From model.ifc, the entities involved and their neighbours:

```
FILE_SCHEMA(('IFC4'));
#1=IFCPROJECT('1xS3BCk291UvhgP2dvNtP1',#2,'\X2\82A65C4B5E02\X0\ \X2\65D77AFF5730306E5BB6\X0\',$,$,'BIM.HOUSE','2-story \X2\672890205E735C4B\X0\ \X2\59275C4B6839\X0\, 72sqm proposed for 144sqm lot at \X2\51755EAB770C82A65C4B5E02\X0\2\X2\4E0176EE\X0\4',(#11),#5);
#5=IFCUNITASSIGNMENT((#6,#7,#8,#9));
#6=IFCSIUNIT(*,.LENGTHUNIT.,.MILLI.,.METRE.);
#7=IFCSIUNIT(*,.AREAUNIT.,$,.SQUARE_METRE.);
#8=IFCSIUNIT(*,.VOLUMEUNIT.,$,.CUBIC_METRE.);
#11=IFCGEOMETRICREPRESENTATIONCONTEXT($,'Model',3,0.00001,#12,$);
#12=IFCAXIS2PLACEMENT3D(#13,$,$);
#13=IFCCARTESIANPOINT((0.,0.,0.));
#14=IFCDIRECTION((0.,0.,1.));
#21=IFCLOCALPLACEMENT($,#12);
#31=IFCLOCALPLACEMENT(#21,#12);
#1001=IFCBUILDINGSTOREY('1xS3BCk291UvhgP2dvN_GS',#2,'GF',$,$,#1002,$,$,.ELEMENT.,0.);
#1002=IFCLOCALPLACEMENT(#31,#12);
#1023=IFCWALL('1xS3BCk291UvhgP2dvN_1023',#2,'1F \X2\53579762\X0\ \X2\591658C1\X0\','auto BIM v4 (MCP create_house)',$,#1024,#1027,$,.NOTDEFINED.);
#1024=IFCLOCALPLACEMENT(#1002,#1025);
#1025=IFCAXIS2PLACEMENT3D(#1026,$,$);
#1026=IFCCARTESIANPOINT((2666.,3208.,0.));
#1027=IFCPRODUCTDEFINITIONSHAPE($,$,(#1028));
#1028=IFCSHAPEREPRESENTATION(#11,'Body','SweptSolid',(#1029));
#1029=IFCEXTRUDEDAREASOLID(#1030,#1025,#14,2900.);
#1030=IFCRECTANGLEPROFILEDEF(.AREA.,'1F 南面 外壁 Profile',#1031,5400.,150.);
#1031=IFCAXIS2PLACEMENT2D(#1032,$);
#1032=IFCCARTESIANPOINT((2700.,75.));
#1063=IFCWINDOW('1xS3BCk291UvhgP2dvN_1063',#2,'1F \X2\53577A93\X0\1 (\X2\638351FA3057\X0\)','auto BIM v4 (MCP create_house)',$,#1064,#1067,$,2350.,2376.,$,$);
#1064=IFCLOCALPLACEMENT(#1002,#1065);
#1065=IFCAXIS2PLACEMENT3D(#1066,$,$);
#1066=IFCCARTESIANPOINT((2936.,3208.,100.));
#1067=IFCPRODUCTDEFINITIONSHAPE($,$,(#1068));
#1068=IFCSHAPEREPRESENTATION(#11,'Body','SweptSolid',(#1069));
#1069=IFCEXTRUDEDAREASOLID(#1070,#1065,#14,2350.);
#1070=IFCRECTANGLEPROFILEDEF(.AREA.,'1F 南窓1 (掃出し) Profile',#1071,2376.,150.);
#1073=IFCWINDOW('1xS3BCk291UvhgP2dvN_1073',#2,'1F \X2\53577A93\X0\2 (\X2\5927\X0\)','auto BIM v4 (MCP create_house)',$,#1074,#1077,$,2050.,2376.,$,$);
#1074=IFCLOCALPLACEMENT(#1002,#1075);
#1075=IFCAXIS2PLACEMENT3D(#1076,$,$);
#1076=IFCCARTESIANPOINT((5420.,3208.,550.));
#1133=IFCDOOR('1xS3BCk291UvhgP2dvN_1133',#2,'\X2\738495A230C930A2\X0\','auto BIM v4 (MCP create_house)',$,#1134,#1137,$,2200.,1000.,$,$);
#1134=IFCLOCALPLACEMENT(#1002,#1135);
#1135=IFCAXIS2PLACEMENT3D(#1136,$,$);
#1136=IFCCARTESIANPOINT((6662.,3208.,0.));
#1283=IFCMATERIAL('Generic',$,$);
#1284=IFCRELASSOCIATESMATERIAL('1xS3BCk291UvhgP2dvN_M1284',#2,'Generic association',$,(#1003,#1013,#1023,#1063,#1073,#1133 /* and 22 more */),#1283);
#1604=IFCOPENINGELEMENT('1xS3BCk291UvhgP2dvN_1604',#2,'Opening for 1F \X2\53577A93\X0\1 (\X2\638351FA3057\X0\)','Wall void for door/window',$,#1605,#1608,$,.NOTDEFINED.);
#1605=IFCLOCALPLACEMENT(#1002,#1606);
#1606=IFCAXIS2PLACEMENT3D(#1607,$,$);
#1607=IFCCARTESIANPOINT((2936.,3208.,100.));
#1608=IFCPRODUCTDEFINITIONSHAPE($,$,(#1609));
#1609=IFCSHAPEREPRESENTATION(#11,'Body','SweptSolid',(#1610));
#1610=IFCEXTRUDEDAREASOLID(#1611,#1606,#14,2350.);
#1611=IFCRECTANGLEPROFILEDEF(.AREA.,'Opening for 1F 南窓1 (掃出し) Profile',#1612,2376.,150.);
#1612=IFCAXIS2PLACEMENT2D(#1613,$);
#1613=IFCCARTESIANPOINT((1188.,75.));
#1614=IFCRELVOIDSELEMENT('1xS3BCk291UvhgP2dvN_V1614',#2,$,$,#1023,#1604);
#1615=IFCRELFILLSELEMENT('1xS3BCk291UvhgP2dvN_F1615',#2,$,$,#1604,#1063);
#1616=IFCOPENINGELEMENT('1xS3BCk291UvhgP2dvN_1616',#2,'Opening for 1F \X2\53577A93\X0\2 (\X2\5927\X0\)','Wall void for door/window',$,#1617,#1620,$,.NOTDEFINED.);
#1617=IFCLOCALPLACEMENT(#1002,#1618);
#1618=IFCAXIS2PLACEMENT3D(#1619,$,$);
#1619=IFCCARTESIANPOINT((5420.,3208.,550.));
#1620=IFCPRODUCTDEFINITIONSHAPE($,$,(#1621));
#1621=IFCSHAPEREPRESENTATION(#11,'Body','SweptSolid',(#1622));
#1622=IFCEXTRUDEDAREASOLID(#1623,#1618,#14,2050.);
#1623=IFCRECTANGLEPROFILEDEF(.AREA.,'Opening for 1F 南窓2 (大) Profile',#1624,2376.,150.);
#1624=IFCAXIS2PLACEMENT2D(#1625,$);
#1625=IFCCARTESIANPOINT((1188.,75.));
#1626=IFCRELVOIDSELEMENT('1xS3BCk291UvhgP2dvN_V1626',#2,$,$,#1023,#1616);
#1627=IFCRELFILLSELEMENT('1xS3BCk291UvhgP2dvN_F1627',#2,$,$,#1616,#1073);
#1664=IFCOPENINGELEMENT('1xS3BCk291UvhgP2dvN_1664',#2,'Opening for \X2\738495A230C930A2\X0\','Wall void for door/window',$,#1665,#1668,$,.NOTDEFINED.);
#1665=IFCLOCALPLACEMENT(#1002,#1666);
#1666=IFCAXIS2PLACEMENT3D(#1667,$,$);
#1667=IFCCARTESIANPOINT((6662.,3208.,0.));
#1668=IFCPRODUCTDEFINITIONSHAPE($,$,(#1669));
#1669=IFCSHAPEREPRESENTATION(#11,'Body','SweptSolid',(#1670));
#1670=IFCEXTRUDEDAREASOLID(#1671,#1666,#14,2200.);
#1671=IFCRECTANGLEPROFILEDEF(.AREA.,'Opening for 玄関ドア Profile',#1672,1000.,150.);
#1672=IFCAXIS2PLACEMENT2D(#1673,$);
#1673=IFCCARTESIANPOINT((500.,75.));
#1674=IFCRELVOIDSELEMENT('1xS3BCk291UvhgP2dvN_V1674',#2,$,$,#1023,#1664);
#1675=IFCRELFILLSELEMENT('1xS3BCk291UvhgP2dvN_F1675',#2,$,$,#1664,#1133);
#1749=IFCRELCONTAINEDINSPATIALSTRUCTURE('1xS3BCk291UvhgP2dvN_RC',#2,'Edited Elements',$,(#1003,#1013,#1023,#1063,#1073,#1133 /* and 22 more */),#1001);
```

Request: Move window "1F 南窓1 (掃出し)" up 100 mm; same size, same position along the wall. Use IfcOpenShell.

```python
import numpy as np
import ifcopenshell
import ifcopenshell.api.geometry
import ifcopenshell.util.placement
import ifcopenshell.util.unit

model = ifcopenshell.open("model.ifc")
unit_scale = ifcopenshell.util.unit.calculate_unit_scale(model)

window = model.by_id(1063)
opening = window.FillsVoids[0].RelatingOpeningElement
dz = 0.1 / unit_scale

shift = np.array([0.0, 0.0, dz])
# The window is not placed relative to its opening, so move both.
for product in (opening, window):
    matrix = ifcopenshell.util.placement.get_local_placement(product.ObjectPlacement)
    matrix[:3, 3] += shift
    ifcopenshell.api.geometry.edit_object_placement(model, product=product, matrix=matrix, is_si=False)

print(f"moved by {dz * unit_scale:+.3f} m")

model.write("model_edited.ifc")
```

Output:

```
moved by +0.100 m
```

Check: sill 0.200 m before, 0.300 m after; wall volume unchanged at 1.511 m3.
